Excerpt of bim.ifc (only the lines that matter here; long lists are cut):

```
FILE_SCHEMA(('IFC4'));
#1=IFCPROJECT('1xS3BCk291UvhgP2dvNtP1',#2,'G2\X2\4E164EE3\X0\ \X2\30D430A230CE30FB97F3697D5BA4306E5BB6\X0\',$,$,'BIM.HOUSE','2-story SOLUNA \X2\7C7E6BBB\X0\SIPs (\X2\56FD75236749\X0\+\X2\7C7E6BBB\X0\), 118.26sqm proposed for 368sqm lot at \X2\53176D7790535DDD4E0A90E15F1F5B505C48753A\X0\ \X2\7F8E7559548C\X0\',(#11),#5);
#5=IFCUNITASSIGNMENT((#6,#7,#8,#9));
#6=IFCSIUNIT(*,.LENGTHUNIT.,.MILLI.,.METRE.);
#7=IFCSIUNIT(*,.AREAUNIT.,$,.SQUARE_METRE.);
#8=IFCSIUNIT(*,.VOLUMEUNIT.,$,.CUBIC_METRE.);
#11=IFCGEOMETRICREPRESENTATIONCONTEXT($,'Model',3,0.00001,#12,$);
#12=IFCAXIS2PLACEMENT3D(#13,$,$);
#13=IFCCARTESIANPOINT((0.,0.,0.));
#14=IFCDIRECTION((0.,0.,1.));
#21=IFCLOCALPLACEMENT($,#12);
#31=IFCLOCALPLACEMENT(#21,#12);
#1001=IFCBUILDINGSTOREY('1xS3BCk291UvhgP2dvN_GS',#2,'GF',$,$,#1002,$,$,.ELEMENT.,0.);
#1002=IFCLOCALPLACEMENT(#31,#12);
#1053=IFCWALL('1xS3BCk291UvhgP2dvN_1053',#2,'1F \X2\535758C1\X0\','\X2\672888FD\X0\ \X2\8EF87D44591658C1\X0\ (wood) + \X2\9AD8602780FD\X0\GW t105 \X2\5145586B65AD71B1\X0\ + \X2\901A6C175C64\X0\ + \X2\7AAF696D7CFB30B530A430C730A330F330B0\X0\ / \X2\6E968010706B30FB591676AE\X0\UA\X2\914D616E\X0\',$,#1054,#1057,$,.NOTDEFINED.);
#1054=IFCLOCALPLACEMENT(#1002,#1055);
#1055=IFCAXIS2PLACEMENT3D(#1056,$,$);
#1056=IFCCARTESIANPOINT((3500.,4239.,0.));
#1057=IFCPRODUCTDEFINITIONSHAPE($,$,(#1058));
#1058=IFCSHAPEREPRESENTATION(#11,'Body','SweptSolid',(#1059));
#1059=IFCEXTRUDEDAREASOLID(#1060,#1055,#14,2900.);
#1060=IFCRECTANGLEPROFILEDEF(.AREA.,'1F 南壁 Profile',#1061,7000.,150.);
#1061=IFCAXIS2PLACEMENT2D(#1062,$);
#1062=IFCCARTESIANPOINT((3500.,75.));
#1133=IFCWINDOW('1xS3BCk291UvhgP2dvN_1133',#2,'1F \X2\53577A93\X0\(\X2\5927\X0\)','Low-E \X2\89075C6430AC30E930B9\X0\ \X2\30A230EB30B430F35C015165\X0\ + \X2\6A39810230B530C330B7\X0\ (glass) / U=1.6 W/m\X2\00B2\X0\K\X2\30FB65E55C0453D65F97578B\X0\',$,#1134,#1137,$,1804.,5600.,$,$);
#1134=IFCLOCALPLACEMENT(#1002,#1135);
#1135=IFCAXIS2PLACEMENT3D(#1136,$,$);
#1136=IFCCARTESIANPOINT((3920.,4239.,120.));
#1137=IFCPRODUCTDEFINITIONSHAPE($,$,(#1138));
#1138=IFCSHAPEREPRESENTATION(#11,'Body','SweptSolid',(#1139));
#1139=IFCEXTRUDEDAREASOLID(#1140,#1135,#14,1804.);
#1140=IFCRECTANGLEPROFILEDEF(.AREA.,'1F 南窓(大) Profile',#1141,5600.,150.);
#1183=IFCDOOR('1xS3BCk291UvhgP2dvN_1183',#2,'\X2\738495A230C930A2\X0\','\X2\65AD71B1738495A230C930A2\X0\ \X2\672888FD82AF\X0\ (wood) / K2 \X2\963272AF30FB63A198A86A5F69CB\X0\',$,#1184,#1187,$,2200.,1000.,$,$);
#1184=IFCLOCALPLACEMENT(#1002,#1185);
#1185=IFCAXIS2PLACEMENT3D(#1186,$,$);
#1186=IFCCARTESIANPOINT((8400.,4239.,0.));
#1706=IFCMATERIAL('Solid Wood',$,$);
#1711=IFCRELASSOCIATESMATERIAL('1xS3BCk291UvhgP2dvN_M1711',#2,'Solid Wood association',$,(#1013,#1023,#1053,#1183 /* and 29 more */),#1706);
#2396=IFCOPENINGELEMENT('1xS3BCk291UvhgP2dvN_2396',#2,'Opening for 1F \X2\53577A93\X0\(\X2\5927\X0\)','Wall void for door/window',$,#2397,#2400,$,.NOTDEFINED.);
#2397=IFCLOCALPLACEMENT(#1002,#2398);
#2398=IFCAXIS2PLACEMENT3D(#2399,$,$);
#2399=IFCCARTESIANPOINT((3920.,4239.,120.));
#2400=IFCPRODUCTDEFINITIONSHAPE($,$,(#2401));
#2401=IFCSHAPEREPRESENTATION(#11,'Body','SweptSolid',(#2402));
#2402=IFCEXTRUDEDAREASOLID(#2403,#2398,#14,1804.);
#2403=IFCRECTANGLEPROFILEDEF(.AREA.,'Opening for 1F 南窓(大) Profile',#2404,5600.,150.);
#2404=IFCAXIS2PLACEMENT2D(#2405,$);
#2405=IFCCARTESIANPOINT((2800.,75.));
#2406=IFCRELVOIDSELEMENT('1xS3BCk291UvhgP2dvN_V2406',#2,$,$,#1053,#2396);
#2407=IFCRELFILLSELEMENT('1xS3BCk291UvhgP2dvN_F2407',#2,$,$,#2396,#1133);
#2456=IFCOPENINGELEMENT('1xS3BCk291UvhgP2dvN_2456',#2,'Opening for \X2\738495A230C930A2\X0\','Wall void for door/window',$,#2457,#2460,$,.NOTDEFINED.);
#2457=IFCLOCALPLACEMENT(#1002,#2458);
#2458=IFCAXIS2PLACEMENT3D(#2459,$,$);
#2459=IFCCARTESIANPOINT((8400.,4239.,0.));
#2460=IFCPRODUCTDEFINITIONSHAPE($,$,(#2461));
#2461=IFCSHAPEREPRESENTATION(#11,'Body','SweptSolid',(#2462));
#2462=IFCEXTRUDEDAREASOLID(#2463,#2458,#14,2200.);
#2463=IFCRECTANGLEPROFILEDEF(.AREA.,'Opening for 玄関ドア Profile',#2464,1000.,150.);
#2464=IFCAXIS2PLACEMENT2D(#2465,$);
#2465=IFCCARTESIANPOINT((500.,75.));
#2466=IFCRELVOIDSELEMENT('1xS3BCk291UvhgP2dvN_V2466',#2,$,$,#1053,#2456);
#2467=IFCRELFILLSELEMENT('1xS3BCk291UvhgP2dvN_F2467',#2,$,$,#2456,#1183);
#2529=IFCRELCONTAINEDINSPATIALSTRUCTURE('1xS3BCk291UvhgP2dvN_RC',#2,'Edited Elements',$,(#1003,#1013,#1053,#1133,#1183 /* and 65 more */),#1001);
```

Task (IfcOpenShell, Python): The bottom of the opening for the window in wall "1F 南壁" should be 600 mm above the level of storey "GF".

```python
import numpy as np
import ifcopenshell
import ifcopenshell.api.geometry
import ifcopenshell.geom
import ifcopenshell.util.element
import ifcopenshell.util.placement
import ifcopenshell.util.shape
import ifcopenshell.util.unit

model = ifcopenshell.open("bim.ifc")
unit_scale = ifcopenshell.util.unit.calculate_unit_scale(model)

window = model.by_guid("1xS3BCk291UvhgP2dvN_1133")
opening = window.FillsVoids[0].RelatingOpeningElement
storey = ifcopenshell.util.element.get_container(window, ifc_class="IfcBuildingStorey")
level = ifcopenshell.util.placement.get_local_placement(storey.ObjectPlacement)[2, 3]

# The opening's origin need not be at the sill, so measure its lowest point.
shape = ifcopenshell.geom.create_shape(ifcopenshell.geom.settings(), opening)
bottom = ifcopenshell.util.shape.get_shape_bottom_elevation(shape, shape.geometry) / unit_scale
dz = level + 600.0 - bottom

shift = np.array([0.0, 0.0, dz])
# The window is not placed relative to its opening, so move both.
for product in (opening, window):
    matrix = ifcopenshell.util.placement.get_local_placement(product.ObjectPlacement)
    matrix[:3, 3] += shift
    ifcopenshell.api.geometry.edit_object_placement(model, product=product, matrix=matrix, is_si=False)

print(f"moved by {dz * unit_scale:+.3f} m")

model.write("bim_updated.ifc")
```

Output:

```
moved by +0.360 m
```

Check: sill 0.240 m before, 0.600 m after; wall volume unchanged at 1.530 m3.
